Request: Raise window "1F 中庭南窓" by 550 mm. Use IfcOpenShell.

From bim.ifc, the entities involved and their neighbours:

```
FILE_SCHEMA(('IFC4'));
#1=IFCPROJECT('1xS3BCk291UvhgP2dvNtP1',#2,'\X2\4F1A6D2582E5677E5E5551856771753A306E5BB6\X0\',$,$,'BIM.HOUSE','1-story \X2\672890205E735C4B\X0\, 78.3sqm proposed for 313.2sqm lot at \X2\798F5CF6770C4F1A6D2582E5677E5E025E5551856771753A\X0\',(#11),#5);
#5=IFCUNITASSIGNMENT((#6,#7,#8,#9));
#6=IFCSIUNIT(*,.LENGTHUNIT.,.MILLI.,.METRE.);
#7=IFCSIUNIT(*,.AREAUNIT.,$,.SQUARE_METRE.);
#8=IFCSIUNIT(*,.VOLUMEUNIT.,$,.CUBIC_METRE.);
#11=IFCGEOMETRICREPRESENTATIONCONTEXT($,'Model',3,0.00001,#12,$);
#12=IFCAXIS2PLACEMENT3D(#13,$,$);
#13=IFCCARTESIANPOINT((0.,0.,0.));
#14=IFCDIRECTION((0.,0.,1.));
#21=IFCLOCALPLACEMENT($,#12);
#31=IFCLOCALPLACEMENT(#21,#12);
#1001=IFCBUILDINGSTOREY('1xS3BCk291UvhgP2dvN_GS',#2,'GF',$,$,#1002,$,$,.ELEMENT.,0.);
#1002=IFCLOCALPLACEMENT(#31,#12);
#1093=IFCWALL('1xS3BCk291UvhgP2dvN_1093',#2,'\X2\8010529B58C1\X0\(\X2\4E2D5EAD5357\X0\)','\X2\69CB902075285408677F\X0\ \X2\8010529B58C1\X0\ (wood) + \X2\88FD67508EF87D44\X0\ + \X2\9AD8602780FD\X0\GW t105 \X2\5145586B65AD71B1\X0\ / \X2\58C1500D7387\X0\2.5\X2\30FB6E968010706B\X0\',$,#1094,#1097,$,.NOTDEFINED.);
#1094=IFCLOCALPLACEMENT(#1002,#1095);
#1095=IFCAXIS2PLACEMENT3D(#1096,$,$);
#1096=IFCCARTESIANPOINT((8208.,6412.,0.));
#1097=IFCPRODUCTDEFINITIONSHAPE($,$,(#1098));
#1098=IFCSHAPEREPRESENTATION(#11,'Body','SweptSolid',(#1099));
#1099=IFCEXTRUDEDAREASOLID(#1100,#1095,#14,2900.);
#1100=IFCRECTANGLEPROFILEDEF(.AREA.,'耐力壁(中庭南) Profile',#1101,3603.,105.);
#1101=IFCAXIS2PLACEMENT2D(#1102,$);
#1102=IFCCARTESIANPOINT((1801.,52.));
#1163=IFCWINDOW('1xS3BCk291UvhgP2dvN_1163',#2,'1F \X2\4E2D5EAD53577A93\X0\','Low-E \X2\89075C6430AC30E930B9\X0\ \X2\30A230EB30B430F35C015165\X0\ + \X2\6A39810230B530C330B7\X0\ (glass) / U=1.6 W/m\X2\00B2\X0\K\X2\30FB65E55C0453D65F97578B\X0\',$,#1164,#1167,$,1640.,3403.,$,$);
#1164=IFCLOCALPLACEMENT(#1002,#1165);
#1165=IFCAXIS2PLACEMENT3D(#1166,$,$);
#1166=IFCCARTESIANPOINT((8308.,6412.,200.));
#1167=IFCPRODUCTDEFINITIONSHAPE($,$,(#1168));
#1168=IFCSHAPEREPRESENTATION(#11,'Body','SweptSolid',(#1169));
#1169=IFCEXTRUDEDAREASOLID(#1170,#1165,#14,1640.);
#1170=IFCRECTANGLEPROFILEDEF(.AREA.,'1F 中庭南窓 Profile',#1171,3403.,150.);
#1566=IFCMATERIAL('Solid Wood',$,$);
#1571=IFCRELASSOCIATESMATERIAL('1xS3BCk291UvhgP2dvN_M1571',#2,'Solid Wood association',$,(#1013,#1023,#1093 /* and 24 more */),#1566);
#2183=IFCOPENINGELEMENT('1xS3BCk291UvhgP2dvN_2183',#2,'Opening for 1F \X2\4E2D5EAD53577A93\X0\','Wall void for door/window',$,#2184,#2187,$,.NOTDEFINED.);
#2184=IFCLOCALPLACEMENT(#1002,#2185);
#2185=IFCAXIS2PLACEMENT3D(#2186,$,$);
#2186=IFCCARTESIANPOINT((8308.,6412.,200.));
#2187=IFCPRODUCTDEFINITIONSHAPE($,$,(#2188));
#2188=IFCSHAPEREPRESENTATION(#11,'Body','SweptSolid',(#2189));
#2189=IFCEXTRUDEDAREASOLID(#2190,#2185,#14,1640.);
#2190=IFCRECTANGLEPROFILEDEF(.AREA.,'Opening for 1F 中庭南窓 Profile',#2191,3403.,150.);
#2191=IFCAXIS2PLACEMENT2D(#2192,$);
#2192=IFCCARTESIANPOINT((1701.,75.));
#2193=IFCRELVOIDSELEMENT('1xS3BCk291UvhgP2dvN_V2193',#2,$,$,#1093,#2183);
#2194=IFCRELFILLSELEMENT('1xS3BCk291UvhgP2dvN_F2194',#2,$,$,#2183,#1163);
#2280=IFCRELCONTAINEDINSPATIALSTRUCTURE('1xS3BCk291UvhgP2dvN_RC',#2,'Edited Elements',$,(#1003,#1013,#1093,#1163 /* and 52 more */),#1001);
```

```python
import numpy as np
import ifcopenshell
import ifcopenshell.api.geometry
import ifcopenshell.util.placement
import ifcopenshell.util.unit

model = ifcopenshell.open("bim.ifc")
unit_scale = ifcopenshell.util.unit.calculate_unit_scale(model)

window = model.by_guid("1xS3BCk291UvhgP2dvN_1163")
opening = window.FillsVoids[0].RelatingOpeningElement
dz = 0.55 / unit_scale

shift = np.array([0.0, 0.0, dz])
# The window is not placed relative to its opening, so move both.
for product in (opening, window):
    matrix = ifcopenshell.util.placement.get_local_placement(product.ObjectPlacement)
    matrix[:3, 3] += shift
    ifcopenshell.api.geometry.edit_object_placement(model, product=product, matrix=matrix, is_si=False)

print(f"moved by {dz * unit_scale:+.3f} m")

model.write("bim_edited.ifc")
```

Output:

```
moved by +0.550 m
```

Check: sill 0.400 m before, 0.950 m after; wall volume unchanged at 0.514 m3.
